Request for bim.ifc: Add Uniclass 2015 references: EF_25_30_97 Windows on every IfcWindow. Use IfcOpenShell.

First a look at what the model holds.

```python
import ifcopenshell

model = ifcopenshell.open("bim.ifc")
print(model.schema)
print("classifications:", [c.Name for c in model.by_type("IfcClassification")])
for ifc_class in ("IfcDoor", "IfcRoof", "IfcStair", "IfcWall", "IfcWindow"):
    print(ifc_class, len(model.by_type(ifc_class)))
```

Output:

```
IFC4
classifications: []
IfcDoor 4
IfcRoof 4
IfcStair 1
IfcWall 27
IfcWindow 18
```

```python
import ifcopenshell
import ifcopenshell.api.classification

model = ifcopenshell.open("bim.ifc")

system = ifcopenshell.api.classification.add_classification(model, classification="Uniclass 2015")

codes = {
    "IfcWindow": ("EF_25_30_97", "Windows"),
}
for ifc_class, (code, name) in codes.items():
    products = model.by_type(ifc_class)
    ifcopenshell.api.classification.add_reference(
        model, products=products, classification=system, identification=code, name=name
    )
    print(code, len(products))

model.write("bim-out.ifc")
```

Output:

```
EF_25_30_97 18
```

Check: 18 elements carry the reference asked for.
